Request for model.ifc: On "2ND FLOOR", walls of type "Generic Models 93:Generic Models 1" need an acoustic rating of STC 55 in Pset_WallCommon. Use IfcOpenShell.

First a look at what the model holds.

```python
import ifcopenshell
import ifcopenshell.util.element

model = ifcopenshell.open("model.ifc")
print(model.schema)
storey = next(s for s in model.by_type("IfcBuildingStorey") if s.Name == "2ND FLOOR")
walls = [e for e in ifcopenshell.util.element.get_decomposition(storey) if e.is_a("IfcWall")]
seen = {}
for e in walls:
    element_type = ifcopenshell.util.element.get_type(e)
    key = (element_type.Name if element_type != e and element_type else None, ifcopenshell.util.element.get_pset(e, "Pset_WallCommon", "AcousticRating"))
    seen[key] = seen.get(key, 0) + 1
for (name, value), count in sorted(seen.items(), key=str):
    print(count, "x", name, "|", value)
```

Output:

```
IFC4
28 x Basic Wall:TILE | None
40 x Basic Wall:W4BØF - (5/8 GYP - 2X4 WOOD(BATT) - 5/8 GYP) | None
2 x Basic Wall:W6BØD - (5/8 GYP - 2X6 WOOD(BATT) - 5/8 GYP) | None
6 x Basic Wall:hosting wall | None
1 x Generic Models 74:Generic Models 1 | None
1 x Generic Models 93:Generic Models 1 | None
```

```python
import ifcopenshell
import ifcopenshell.api.pset
import ifcopenshell.util.element

model = ifcopenshell.open("model.ifc")

storey = next(s for s in model.by_type("IfcBuildingStorey") if s.Name == "2ND FLOOR")
walls = [e for e in ifcopenshell.util.element.get_decomposition(storey) if e.is_a("IfcWall")]

count = 0
for e in walls:
    element_type = ifcopenshell.util.element.get_type(e)
    if element_type in (None, e) or element_type.Name != "Generic Models 93:Generic Models 1":
        continue
    # add_pset returns the element's existing set when there is one.
    pset = ifcopenshell.api.pset.add_pset(model, product=e, name="Pset_WallCommon")
    ifcopenshell.api.pset.edit_pset(model, pset=pset, properties={"AcousticRating": "STC 55"})
    count += 1

print(count, "walls updated")

model.write("model_edited.ifc")
```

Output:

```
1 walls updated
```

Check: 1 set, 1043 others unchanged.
